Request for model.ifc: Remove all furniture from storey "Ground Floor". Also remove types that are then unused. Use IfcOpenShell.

First a look at what the model holds.

```python
import ifcopenshell
import ifcopenshell.util.element

model = ifcopenshell.open("model.ifc")
print(model.schema)
storey = next(s for s in model.by_type("IfcBuildingStorey") if s.Name == "Ground Floor")
furniture = [e for e in ifcopenshell.util.element.get_decomposition(storey) if e.is_a("IfcFurnishingElement")]
seen = {}
for e in furniture:
    element_type = ifcopenshell.util.element.get_type(e)
    name = element_type.Name if element_type not in (None, e) else None
    seen[name] = seen.get(name, 0) + 1
for name, count in sorted(seen.items(), key=str):
    print(count, "x", name)
```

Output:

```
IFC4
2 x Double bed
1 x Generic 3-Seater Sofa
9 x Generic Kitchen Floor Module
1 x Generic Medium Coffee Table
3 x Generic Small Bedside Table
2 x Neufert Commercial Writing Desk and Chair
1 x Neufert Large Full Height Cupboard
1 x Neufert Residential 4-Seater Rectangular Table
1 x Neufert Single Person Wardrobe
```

```python
import ifcopenshell
import ifcopenshell.api.root
import ifcopenshell.util.element

model = ifcopenshell.open("model.ifc")

storey = next(s for s in model.by_type("IfcBuildingStorey") if s.Name == "Ground Floor")
furniture = [e for e in ifcopenshell.util.element.get_decomposition(storey) if e.is_a("IfcFurnishingElement")]
types = {ifcopenshell.util.element.get_type(e) for e in furniture} - {None, *furniture}

for e in furniture:
    ifcopenshell.api.root.remove_product(model, product=e)
print(len(furniture), "removed")

unused = [t for t in types if not ifcopenshell.util.element.get_types(t)]
for t in unused:
    ifcopenshell.api.root.remove_product(model, product=t)
print(len(unused), "unused types removed")

model.write("model_edited.ifc")
```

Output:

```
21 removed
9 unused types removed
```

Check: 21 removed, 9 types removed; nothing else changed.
